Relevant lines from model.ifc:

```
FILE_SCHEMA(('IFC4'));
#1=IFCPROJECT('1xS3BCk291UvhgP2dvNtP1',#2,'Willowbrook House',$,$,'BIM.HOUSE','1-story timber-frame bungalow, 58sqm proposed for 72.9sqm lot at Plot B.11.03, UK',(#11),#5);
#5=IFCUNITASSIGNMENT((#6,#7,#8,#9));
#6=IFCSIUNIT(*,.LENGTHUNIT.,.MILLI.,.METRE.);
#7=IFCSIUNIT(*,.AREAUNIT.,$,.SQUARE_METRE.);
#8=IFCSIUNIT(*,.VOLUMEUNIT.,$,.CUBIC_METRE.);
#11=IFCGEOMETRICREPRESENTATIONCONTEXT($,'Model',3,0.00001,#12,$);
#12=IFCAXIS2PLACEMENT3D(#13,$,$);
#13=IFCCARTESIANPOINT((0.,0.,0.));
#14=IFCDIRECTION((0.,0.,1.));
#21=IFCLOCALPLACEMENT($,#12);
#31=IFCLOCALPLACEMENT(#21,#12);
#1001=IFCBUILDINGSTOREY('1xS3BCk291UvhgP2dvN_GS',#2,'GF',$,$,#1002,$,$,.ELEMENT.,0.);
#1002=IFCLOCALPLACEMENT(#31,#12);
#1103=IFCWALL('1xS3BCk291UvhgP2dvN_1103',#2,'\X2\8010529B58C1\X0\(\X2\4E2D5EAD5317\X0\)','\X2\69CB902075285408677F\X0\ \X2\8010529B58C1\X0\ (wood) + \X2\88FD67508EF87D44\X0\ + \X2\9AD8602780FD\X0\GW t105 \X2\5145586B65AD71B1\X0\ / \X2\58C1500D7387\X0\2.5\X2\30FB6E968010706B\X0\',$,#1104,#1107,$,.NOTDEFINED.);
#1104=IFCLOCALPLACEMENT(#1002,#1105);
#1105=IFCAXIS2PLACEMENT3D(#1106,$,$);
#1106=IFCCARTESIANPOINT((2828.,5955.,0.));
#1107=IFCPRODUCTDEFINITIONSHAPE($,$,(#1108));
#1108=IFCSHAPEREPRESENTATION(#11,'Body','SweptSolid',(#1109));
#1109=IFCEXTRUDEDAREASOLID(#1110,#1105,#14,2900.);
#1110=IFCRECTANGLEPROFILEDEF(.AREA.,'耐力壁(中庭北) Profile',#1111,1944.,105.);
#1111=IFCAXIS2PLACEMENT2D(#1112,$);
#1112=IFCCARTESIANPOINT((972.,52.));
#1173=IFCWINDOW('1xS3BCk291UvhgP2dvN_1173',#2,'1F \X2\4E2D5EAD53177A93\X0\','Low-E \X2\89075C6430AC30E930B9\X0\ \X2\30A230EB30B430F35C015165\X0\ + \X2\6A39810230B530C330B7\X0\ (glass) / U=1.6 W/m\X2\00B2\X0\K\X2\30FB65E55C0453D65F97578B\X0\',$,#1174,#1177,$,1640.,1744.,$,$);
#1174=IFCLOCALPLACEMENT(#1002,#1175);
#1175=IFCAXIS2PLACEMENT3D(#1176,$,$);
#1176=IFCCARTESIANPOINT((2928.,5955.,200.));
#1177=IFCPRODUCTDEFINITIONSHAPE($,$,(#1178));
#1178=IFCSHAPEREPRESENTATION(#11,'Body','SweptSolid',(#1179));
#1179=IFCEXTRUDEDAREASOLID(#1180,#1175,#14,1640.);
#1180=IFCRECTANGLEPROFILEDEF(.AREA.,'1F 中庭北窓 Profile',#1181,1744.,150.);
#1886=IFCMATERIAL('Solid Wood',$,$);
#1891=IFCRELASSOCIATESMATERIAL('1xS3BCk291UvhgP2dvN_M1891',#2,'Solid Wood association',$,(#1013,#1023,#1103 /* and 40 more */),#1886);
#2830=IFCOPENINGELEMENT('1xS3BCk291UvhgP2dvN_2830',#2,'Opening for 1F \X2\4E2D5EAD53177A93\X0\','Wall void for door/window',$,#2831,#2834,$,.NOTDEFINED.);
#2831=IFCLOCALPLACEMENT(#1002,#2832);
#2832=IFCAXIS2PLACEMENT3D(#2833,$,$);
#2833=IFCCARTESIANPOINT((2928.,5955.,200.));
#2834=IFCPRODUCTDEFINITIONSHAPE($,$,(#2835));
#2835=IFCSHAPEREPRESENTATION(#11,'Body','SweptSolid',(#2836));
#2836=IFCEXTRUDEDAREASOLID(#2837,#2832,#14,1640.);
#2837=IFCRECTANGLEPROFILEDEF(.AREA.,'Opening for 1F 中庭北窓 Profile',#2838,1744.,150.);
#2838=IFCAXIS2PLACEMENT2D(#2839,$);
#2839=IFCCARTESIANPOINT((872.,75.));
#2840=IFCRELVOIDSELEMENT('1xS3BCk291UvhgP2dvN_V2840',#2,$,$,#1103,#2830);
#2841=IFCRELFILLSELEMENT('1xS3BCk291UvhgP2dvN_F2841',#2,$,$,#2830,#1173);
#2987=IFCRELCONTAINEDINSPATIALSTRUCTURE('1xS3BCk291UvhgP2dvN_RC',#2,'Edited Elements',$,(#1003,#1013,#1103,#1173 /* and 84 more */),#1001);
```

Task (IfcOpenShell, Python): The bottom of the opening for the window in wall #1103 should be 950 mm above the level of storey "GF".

```python
import numpy as np
import ifcopenshell
import ifcopenshell.api.geometry
import ifcopenshell.geom
import ifcopenshell.util.element
import ifcopenshell.util.placement
import ifcopenshell.util.shape
import ifcopenshell.util.unit

model = ifcopenshell.open("model.ifc")
unit_scale = ifcopenshell.util.unit.calculate_unit_scale(model)

window = model.by_guid("1xS3BCk291UvhgP2dvN_1173")
opening = window.FillsVoids[0].RelatingOpeningElement
storey = ifcopenshell.util.element.get_container(window, ifc_class="IfcBuildingStorey")
level = ifcopenshell.util.placement.get_local_placement(storey.ObjectPlacement)[2, 3]

# The opening's origin need not be at the sill, so measure its lowest point.
shape = ifcopenshell.geom.create_shape(ifcopenshell.geom.settings(), opening)
bottom = ifcopenshell.util.shape.get_shape_bottom_elevation(shape, shape.geometry) / unit_scale
dz = level + 0.95 / unit_scale - bottom

shift = np.array([0.0, 0.0, dz])
# The window is not placed relative to its opening, so move both.
for product in (opening, window):
    matrix = ifcopenshell.util.placement.get_local_placement(product.ObjectPlacement)
    matrix[:3, 3] += shift
    ifcopenshell.api.geometry.edit_object_placement(model, product=product, matrix=matrix, is_si=False)

print(f"moved by {dz * unit_scale:+.3f} m")

model.write("model_rev.ifc")
```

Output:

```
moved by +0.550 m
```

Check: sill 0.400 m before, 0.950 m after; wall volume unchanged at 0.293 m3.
